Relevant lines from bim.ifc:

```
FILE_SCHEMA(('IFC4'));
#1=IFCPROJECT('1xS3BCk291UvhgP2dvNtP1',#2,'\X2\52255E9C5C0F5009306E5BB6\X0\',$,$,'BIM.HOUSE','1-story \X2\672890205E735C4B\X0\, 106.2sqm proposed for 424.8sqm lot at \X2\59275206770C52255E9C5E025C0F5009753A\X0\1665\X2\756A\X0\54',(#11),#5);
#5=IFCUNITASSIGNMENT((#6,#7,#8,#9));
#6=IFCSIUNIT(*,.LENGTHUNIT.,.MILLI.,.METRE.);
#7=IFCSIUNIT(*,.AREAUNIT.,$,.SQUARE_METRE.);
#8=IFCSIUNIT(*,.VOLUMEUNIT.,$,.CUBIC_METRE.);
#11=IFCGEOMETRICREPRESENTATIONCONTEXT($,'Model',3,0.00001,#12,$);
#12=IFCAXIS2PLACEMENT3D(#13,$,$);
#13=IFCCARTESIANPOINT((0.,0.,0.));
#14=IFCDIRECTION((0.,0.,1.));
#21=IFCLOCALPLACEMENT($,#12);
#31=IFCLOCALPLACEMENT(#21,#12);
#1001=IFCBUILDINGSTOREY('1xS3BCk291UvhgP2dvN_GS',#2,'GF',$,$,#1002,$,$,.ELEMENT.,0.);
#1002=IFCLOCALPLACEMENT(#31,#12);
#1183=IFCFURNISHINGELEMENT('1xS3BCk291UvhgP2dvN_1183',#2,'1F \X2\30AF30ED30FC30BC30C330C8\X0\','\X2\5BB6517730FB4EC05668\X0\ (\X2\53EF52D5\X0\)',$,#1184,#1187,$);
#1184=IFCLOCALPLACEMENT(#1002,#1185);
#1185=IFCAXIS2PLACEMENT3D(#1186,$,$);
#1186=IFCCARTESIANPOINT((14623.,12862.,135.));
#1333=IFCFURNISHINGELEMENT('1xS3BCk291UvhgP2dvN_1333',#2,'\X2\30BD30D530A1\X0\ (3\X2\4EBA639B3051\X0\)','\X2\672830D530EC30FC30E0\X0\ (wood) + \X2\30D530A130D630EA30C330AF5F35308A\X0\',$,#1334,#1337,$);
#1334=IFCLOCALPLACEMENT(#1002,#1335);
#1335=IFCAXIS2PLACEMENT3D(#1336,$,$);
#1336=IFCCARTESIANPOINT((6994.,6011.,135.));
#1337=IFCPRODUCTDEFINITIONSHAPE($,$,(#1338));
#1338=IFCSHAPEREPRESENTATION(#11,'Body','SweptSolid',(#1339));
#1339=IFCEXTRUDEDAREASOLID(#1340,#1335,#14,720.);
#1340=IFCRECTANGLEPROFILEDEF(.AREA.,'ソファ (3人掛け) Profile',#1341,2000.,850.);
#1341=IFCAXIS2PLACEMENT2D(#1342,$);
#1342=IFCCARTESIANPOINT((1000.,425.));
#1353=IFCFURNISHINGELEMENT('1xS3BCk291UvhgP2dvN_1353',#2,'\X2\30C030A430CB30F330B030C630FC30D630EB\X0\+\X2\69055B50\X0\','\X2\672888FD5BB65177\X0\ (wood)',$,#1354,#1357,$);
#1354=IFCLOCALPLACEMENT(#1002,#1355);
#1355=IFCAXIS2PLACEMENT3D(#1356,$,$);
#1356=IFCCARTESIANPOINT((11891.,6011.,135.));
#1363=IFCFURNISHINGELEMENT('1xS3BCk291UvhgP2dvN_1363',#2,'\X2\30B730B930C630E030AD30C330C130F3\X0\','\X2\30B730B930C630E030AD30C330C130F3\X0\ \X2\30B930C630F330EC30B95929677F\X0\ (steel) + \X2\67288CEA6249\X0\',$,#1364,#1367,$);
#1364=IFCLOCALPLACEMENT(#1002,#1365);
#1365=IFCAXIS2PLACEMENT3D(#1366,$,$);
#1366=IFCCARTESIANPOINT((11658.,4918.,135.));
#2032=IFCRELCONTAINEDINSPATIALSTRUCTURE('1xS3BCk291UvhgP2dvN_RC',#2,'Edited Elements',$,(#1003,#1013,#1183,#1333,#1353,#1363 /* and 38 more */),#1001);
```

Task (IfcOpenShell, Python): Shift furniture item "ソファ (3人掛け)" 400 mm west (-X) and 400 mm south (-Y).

```python
import ifcopenshell
import ifcopenshell.api.geometry
import ifcopenshell.util.placement
import ifcopenshell.util.unit

model = ifcopenshell.open("bim.ifc")
unit_scale = ifcopenshell.util.unit.calculate_unit_scale(model)

item = model.by_guid("1xS3BCk291UvhgP2dvN_1333")
matrix = ifcopenshell.util.placement.get_local_placement(item.ObjectPlacement)
matrix[0, 3] -= 0.4 / unit_scale
matrix[1, 3] -= 0.4 / unit_scale
ifcopenshell.api.geometry.edit_object_placement(model, product=item, matrix=matrix, is_si=False)

print(ifcopenshell.util.placement.get_local_placement(item.ObjectPlacement).round(3) + 0.0)

model.write("bim_updated.ifc")
```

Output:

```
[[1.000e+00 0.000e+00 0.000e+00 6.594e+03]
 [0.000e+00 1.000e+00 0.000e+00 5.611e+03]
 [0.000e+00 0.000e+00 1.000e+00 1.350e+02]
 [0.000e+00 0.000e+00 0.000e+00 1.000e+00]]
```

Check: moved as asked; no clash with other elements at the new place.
